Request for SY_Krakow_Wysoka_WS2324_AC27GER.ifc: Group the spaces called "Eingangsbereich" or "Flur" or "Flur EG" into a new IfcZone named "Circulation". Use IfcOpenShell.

First a look at what the model holds.

```python
import ifcopenshell

model = ifcopenshell.open("SY_Krakow_Wysoka_WS2324_AC27GER.ifc")
print(model.schema)
seen = {}
for space in model.by_type("IfcSpace"):
    seen[space.LongName] = seen.get(space.LongName, 0) + 1
for name, count in sorted(seen.items(), key=str):
    print(count, "x", name)
print("zones:", [z.Name for z in model.by_type("IfcZone")][:20])
```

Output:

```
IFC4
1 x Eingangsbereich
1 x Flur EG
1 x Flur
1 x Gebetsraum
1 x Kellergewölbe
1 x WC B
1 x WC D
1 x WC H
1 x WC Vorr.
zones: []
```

```python
import ifcopenshell
import ifcopenshell.api.group
import ifcopenshell.api.root

model = ifcopenshell.open("SY_Krakow_Wysoka_WS2324_AC27GER.ifc")

names = {"Eingangsbereich", "Flur", "Flur EG"}
spaces = [s for s in model.by_type("IfcSpace") if s.LongName in names]

zone = ifcopenshell.api.root.create_entity(model, ifc_class="IfcZone", name="Circulation")
ifcopenshell.api.group.assign_group(model, products=spaces, group=zone)
print(len(spaces), "spaces in", zone.Name)

model.write("SY_Krakow_Wysoka_WS2324_AC27GER_rev.ifc")
```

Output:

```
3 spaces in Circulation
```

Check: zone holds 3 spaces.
